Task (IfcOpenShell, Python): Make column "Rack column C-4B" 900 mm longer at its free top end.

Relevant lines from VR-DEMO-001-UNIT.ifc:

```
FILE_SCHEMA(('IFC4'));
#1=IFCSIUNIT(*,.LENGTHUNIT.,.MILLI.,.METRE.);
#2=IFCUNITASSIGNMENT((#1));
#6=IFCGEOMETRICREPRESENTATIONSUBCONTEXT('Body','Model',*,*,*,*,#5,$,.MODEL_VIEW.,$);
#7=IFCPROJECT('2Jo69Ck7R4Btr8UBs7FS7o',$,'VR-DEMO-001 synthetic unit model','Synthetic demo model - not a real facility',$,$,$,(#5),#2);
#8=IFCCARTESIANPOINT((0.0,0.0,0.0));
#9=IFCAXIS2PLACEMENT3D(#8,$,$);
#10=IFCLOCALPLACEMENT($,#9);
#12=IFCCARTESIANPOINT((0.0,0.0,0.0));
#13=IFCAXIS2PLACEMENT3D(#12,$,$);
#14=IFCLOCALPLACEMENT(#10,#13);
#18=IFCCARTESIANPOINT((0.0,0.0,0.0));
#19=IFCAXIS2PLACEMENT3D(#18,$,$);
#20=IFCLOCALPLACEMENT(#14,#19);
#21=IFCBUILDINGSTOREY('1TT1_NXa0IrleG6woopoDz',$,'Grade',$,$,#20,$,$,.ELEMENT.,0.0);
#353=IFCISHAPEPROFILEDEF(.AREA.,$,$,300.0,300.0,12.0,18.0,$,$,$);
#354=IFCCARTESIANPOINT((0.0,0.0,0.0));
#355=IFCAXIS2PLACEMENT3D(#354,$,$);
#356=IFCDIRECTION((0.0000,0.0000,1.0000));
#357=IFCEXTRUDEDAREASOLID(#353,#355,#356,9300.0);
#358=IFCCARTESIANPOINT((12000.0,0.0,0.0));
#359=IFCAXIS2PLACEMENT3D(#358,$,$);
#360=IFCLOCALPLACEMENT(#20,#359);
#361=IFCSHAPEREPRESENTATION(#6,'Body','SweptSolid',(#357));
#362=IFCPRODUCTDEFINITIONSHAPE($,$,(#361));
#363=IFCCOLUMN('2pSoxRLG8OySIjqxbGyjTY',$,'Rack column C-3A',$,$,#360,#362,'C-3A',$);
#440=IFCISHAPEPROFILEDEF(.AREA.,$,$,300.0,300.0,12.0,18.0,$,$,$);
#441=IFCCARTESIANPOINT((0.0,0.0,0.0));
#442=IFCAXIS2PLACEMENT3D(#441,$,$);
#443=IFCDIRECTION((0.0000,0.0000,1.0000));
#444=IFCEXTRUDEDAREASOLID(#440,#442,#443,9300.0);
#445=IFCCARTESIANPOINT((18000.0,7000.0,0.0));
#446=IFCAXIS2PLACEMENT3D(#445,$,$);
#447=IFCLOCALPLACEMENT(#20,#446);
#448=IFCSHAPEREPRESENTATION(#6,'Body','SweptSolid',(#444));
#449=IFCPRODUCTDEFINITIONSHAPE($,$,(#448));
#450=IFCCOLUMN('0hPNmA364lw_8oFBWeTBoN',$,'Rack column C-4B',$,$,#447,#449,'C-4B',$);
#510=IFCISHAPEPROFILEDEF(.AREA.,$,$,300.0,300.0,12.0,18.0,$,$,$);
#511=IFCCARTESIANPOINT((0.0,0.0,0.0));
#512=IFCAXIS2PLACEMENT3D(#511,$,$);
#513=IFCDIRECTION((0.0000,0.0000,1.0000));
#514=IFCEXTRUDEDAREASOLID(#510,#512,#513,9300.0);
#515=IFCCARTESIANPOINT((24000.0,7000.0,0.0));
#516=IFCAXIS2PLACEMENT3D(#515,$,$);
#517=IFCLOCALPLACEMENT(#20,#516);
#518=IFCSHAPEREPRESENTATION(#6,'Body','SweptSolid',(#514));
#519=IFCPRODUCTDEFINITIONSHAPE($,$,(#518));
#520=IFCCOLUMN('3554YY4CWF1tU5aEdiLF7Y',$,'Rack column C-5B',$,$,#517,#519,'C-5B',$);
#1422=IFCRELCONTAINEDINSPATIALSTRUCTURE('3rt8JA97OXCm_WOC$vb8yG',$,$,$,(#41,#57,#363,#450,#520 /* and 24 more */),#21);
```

```python
import ifcopenshell
import ifcopenshell.util.representation

model = ifcopenshell.open("VR-DEMO-001-UNIT.ifc")

member = model.by_id(450)
change = 900.0

# The extrusion runs towards the end named, so only its depth changes.
body = ifcopenshell.util.representation.get_representation(member, "Model", "Body")
solid = body.Items[0]
old_length = solid.Depth
solid.Depth += change

print(f"length {old_length:g} -> {solid.Depth:g}")

model.write("VR-DEMO-001-UNIT_rev.ifc")
```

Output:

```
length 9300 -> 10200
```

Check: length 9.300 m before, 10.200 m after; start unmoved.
